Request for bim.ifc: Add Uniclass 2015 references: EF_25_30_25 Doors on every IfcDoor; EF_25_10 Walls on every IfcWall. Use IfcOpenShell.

First a look at what the model holds.

```python
import ifcopenshell

model = ifcopenshell.open("bim.ifc")
print(model.schema)
print("classifications:", [c.Name for c in model.by_type("IfcClassification")])
for ifc_class in ("IfcDoor", "IfcRoof", "IfcStair", "IfcWall", "IfcWindow"):
    print(ifc_class, len(model.by_type(ifc_class)))
```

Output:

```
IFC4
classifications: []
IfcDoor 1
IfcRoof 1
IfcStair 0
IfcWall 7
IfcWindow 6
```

```python
import ifcopenshell
import ifcopenshell.api.classification

model = ifcopenshell.open("bim.ifc")

system = ifcopenshell.api.classification.add_classification(model, classification="Uniclass 2015")

codes = {
    "IfcDoor": ("EF_25_30_25", "Doors"),
    "IfcWall": ("EF_25_10", "Walls"),
}
for ifc_class, (code, name) in codes.items():
    products = model.by_type(ifc_class)
    ifcopenshell.api.classification.add_reference(
        model, products=products, classification=system, identification=code, name=name
    )
    print(code, len(products))

model.write("bim_edited.ifc")
```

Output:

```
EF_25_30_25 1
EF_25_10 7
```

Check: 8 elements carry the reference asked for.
